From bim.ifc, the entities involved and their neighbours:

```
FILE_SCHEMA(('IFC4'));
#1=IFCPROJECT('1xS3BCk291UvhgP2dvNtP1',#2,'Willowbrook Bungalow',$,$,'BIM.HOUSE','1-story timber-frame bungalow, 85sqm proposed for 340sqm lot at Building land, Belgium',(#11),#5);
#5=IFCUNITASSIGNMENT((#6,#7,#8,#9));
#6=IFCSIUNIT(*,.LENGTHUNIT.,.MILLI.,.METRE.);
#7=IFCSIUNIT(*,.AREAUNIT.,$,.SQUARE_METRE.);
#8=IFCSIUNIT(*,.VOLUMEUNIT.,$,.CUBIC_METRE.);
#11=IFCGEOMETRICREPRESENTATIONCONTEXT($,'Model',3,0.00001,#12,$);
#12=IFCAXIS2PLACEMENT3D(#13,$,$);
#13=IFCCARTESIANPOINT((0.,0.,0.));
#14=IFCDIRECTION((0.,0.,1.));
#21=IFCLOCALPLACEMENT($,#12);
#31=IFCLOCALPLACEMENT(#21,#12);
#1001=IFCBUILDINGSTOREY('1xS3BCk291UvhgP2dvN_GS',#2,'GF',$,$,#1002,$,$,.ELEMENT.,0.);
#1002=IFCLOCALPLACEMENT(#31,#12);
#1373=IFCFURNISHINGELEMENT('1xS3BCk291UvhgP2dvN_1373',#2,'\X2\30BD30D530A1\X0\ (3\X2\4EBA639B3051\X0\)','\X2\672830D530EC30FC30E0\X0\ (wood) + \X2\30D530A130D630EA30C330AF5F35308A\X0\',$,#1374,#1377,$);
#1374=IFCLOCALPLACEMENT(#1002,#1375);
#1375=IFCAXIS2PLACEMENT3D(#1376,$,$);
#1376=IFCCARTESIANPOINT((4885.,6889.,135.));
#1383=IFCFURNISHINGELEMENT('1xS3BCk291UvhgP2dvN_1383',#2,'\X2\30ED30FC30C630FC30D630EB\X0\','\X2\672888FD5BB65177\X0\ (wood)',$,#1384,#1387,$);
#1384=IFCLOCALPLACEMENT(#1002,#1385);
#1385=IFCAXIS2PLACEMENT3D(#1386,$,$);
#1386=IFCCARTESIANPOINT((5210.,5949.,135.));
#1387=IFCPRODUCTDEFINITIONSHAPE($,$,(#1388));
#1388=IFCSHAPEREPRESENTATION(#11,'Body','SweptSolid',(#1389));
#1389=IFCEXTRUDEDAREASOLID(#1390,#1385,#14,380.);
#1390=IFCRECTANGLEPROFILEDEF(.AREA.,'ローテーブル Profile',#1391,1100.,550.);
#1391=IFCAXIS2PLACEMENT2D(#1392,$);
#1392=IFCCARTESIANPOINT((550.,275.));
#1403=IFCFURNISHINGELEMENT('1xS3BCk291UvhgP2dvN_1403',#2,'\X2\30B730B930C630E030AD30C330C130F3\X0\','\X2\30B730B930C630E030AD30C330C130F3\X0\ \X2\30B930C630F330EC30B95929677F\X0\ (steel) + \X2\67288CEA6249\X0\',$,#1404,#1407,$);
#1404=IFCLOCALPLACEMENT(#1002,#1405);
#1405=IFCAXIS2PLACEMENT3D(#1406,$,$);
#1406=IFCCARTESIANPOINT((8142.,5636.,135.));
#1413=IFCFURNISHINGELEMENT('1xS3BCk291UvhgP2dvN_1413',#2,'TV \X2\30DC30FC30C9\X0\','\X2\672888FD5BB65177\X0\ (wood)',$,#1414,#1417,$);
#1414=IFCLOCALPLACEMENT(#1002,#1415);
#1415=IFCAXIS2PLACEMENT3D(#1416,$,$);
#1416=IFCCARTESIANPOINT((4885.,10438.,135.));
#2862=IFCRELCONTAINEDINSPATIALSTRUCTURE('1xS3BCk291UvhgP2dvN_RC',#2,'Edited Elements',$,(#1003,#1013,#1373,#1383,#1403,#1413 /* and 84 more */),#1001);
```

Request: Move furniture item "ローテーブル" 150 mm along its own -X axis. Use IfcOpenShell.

```python
import ifcopenshell
import ifcopenshell.api.geometry
import ifcopenshell.util.placement

model = ifcopenshell.open("bim.ifc")

item = model.by_id(1383)
matrix = ifcopenshell.util.placement.get_local_placement(item.ObjectPlacement)
matrix[:3, 3] -= matrix[:3, 0] * 150.0
ifcopenshell.api.geometry.edit_object_placement(model, product=item, matrix=matrix, is_si=False)

print(ifcopenshell.util.placement.get_local_placement(item.ObjectPlacement).round(3) + 0.0)

model.write("bim_v2.ifc")
```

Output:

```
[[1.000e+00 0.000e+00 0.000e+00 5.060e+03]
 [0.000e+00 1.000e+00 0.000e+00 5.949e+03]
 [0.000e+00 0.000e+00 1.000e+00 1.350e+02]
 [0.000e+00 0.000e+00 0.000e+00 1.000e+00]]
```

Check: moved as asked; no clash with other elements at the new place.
